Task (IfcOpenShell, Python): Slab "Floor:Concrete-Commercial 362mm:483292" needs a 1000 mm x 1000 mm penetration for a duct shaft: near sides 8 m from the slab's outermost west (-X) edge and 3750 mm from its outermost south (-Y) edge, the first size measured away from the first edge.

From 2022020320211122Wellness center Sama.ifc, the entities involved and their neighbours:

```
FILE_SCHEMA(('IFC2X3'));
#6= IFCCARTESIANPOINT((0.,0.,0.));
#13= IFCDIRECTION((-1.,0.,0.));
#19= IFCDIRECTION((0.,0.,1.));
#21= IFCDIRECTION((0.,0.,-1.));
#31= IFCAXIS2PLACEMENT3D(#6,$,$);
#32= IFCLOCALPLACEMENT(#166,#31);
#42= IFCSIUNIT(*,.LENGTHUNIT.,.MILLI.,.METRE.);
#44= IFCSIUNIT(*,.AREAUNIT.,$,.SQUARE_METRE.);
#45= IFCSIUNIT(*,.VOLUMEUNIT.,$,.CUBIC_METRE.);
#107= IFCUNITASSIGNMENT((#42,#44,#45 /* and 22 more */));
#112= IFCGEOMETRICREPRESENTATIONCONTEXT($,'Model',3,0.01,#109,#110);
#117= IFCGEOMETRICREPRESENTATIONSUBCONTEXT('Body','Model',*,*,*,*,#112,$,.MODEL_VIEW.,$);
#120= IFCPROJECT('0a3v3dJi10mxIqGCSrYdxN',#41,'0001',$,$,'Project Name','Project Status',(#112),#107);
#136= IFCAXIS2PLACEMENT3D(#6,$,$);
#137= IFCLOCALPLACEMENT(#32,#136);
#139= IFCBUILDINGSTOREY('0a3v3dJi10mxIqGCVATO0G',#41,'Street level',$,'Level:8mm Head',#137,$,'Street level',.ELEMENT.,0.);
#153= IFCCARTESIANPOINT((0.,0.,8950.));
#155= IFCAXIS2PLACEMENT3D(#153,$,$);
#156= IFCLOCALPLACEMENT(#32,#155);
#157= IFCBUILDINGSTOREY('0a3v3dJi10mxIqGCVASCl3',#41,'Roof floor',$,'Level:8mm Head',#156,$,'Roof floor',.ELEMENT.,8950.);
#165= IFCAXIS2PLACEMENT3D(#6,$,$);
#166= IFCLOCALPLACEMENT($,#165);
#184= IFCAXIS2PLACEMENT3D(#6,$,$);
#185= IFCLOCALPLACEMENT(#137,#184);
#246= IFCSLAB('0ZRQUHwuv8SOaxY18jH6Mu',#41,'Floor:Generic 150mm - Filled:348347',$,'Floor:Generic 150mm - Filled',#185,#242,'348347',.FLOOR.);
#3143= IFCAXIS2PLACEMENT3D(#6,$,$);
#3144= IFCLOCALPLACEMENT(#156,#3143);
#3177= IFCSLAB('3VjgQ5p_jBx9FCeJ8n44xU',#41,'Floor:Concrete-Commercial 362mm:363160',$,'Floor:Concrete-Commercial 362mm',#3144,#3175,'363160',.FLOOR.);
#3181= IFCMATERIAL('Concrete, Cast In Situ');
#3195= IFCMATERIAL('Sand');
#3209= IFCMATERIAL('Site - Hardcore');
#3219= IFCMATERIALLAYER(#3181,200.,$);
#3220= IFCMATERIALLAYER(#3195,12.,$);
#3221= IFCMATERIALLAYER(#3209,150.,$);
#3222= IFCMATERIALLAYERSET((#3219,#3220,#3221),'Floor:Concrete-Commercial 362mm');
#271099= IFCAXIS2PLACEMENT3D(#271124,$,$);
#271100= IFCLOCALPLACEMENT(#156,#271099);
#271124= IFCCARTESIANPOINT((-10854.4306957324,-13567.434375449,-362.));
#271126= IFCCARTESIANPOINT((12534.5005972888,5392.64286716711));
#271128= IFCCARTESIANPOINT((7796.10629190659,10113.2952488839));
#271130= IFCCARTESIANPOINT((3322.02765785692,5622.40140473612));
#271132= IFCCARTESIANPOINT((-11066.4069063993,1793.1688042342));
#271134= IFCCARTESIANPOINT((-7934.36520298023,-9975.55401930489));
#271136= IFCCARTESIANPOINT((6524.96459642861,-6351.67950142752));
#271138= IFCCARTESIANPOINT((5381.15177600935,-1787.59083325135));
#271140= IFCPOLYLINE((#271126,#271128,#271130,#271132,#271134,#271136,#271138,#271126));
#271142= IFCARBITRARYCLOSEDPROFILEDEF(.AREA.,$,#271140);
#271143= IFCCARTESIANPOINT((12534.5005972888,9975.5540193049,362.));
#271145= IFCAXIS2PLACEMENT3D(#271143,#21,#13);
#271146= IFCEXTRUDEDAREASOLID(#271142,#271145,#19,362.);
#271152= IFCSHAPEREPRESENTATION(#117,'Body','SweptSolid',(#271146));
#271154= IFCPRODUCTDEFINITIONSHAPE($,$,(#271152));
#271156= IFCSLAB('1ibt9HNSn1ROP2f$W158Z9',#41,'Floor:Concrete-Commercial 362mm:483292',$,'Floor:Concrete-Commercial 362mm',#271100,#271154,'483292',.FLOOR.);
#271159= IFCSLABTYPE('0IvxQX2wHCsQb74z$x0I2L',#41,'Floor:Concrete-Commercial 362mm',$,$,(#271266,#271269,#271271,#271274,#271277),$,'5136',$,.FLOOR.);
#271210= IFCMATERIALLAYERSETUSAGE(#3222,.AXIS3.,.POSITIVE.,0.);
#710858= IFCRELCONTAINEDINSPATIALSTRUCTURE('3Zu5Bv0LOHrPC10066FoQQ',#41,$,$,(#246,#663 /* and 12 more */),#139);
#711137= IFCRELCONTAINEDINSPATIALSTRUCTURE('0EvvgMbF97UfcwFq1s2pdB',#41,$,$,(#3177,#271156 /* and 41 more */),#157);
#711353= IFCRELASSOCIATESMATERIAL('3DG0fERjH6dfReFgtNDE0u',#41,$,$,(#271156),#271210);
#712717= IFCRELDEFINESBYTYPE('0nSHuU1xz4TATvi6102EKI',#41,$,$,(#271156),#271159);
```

```python
import numpy as np
import ifcopenshell
import ifcopenshell.api.feature
import ifcopenshell.api.geometry
import ifcopenshell.api.root
import ifcopenshell.geom
import ifcopenshell.util.placement
import ifcopenshell.util.representation
import ifcopenshell.util.shape
import ifcopenshell.util.unit

model = ifcopenshell.open("2022020320211122Wellness center Sama.ifc")
unit_scale = ifcopenshell.util.unit.calculate_unit_scale(model)
settings = ifcopenshell.geom.settings()


def volume(element):
    """Net volume in cubic metres, openings subtracted."""
    shape = ifcopenshell.geom.create_shape(settings, element)
    return ifcopenshell.util.shape.get_volume(shape.geometry)


slab = model.by_guid("1ibt9HNSn1ROP2f$W158Z9")
before = volume(slab)

# Extent in the slab's own axes, in metres. The edges named are its -X and -Y sides.
slab_shape = ifcopenshell.geom.create_shape(settings, slab)
vertices = ifcopenshell.util.shape.get_vertices(slab_shape.geometry)
x_min, y_min, bottom = vertices.min(axis=0)
top = vertices[:, 2].max()

opening = ifcopenshell.api.root.create_entity(model, ifc_class="IfcOpeningElement", name="Duct shaft opening")
context = ifcopenshell.util.representation.get_context(model, "Model", "Body", "MODEL_VIEW")
width, depth = 1, 1
outline = [(0.0, 0.0), (width, 0.0), (width, depth), (0.0, depth), (0.0, 0.0)]
# Overshoot both faces by 50 mm so the cut is clean.
shape = ifcopenshell.api.geometry.add_slab_representation(
    model, context=context, depth=top - bottom + 0.1, polyline=outline
)
ifcopenshell.api.geometry.assign_representation(model, product=opening, representation=shape)

matrix = ifcopenshell.util.placement.get_local_placement(slab.ObjectPlacement)
matrix[:, 3] = matrix @ np.append(np.array([x_min + 8, y_min + 3.75, bottom - 0.05]) / unit_scale, 1.0)
ifcopenshell.api.geometry.edit_object_placement(model, product=opening, matrix=matrix, is_si=False)
ifcopenshell.api.feature.add_feature(model, feature=opening, element=slab)

after = volume(slab)

print(f"slab volume {before:.3f} -> {after:.3f} m3")

model.write("2022020320211122Wellness center Sama_edited.ifc")
```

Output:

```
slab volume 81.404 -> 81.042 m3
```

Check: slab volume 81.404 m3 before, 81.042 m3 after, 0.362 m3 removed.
